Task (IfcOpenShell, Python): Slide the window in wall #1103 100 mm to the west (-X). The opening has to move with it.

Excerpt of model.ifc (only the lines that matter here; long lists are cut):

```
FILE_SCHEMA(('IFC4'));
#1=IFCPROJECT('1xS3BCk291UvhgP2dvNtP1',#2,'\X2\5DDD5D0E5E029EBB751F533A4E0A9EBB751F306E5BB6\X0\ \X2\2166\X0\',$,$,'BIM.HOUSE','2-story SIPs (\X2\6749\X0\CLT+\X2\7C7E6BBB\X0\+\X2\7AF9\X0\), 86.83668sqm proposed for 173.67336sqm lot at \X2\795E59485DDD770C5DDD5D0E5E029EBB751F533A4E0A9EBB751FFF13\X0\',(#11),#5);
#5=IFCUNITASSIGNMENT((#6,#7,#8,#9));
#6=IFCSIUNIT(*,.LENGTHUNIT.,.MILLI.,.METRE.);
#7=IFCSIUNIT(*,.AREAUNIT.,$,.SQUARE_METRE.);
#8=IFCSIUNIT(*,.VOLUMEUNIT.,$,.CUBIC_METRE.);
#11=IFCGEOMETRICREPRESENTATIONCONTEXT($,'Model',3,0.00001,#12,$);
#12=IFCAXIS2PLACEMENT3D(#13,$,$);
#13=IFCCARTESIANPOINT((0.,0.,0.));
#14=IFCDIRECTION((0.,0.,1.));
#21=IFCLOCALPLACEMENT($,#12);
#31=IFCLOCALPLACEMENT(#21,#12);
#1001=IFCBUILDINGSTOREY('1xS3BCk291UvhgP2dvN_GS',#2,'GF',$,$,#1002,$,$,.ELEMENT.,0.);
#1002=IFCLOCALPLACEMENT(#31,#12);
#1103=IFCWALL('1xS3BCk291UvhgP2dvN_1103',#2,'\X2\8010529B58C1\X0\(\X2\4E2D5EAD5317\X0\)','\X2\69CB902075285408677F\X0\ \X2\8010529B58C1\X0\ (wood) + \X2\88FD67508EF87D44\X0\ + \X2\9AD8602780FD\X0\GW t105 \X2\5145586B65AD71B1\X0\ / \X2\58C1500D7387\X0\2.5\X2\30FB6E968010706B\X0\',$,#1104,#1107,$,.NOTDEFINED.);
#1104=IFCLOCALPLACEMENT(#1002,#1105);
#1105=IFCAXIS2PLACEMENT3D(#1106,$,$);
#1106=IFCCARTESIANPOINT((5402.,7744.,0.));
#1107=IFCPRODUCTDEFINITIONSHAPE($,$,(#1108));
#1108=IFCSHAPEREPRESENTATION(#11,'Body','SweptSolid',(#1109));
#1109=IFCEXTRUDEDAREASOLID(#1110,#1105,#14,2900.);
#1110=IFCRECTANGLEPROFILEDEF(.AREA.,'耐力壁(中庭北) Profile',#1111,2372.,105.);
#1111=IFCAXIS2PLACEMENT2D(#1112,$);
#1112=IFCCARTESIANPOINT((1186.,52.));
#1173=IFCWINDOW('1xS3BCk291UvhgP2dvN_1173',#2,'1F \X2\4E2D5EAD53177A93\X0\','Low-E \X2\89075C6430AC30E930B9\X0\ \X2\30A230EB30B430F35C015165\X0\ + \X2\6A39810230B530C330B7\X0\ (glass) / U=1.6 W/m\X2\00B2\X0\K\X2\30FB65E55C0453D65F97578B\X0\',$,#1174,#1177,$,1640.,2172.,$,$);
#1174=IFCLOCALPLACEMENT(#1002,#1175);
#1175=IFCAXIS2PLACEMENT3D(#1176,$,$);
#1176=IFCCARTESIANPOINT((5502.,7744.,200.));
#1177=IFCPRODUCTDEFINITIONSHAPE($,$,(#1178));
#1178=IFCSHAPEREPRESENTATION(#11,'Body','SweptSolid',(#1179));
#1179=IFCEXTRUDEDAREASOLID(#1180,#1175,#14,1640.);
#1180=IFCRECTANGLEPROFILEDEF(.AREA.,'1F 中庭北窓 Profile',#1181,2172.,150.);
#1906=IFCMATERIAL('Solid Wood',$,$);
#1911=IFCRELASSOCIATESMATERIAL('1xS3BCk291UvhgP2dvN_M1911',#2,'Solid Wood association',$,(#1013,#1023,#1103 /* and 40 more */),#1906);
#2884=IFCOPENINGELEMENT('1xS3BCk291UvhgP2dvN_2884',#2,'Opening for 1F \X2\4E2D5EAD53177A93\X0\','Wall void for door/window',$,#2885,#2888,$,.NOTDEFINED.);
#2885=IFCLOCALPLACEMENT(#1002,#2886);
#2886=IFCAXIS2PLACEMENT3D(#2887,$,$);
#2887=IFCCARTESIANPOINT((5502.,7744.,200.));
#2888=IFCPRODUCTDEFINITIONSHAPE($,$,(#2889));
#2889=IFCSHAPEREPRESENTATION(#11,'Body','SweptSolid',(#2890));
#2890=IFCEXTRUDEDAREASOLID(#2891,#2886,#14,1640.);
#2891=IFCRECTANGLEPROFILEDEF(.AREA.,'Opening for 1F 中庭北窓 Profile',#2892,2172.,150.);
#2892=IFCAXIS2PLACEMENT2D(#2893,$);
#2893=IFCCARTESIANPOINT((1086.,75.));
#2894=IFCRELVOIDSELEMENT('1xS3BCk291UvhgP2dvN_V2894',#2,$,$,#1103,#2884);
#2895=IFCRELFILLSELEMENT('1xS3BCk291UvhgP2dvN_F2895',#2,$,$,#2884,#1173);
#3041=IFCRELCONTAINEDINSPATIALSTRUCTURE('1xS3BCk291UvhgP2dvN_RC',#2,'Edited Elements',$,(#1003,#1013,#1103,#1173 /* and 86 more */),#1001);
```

```python
import ifcopenshell
import ifcopenshell.api.geometry
import ifcopenshell.util.placement

model = ifcopenshell.open("model.ifc")

window = model.by_guid("1xS3BCk291UvhgP2dvN_1173")
opening = window.FillsVoids[0].RelatingOpeningElement
wall = opening.VoidsElements[0].RelatingBuildingElement

wall_matrix = ifcopenshell.util.placement.get_local_placement(wall.ObjectPlacement)
shift = wall_matrix[:3, 0] * -100.0
before = ifcopenshell.util.placement.get_local_placement(window.ObjectPlacement)[:3, 3].copy()

# The window is not placed relative to its opening, so move both.
for product in (opening, window):
    matrix = ifcopenshell.util.placement.get_local_placement(product.ObjectPlacement)
    matrix[:3, 3] += shift
    ifcopenshell.api.geometry.edit_object_placement(model, product=product, matrix=matrix, is_si=False)

after = ifcopenshell.util.placement.get_local_placement(window.ObjectPlacement)[:3, 3]
print("window moved by", (after - before).round(3) + 0.0)

model.write("model-out.ifc")
```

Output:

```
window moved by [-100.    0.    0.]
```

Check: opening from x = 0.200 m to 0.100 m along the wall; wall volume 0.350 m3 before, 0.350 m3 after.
